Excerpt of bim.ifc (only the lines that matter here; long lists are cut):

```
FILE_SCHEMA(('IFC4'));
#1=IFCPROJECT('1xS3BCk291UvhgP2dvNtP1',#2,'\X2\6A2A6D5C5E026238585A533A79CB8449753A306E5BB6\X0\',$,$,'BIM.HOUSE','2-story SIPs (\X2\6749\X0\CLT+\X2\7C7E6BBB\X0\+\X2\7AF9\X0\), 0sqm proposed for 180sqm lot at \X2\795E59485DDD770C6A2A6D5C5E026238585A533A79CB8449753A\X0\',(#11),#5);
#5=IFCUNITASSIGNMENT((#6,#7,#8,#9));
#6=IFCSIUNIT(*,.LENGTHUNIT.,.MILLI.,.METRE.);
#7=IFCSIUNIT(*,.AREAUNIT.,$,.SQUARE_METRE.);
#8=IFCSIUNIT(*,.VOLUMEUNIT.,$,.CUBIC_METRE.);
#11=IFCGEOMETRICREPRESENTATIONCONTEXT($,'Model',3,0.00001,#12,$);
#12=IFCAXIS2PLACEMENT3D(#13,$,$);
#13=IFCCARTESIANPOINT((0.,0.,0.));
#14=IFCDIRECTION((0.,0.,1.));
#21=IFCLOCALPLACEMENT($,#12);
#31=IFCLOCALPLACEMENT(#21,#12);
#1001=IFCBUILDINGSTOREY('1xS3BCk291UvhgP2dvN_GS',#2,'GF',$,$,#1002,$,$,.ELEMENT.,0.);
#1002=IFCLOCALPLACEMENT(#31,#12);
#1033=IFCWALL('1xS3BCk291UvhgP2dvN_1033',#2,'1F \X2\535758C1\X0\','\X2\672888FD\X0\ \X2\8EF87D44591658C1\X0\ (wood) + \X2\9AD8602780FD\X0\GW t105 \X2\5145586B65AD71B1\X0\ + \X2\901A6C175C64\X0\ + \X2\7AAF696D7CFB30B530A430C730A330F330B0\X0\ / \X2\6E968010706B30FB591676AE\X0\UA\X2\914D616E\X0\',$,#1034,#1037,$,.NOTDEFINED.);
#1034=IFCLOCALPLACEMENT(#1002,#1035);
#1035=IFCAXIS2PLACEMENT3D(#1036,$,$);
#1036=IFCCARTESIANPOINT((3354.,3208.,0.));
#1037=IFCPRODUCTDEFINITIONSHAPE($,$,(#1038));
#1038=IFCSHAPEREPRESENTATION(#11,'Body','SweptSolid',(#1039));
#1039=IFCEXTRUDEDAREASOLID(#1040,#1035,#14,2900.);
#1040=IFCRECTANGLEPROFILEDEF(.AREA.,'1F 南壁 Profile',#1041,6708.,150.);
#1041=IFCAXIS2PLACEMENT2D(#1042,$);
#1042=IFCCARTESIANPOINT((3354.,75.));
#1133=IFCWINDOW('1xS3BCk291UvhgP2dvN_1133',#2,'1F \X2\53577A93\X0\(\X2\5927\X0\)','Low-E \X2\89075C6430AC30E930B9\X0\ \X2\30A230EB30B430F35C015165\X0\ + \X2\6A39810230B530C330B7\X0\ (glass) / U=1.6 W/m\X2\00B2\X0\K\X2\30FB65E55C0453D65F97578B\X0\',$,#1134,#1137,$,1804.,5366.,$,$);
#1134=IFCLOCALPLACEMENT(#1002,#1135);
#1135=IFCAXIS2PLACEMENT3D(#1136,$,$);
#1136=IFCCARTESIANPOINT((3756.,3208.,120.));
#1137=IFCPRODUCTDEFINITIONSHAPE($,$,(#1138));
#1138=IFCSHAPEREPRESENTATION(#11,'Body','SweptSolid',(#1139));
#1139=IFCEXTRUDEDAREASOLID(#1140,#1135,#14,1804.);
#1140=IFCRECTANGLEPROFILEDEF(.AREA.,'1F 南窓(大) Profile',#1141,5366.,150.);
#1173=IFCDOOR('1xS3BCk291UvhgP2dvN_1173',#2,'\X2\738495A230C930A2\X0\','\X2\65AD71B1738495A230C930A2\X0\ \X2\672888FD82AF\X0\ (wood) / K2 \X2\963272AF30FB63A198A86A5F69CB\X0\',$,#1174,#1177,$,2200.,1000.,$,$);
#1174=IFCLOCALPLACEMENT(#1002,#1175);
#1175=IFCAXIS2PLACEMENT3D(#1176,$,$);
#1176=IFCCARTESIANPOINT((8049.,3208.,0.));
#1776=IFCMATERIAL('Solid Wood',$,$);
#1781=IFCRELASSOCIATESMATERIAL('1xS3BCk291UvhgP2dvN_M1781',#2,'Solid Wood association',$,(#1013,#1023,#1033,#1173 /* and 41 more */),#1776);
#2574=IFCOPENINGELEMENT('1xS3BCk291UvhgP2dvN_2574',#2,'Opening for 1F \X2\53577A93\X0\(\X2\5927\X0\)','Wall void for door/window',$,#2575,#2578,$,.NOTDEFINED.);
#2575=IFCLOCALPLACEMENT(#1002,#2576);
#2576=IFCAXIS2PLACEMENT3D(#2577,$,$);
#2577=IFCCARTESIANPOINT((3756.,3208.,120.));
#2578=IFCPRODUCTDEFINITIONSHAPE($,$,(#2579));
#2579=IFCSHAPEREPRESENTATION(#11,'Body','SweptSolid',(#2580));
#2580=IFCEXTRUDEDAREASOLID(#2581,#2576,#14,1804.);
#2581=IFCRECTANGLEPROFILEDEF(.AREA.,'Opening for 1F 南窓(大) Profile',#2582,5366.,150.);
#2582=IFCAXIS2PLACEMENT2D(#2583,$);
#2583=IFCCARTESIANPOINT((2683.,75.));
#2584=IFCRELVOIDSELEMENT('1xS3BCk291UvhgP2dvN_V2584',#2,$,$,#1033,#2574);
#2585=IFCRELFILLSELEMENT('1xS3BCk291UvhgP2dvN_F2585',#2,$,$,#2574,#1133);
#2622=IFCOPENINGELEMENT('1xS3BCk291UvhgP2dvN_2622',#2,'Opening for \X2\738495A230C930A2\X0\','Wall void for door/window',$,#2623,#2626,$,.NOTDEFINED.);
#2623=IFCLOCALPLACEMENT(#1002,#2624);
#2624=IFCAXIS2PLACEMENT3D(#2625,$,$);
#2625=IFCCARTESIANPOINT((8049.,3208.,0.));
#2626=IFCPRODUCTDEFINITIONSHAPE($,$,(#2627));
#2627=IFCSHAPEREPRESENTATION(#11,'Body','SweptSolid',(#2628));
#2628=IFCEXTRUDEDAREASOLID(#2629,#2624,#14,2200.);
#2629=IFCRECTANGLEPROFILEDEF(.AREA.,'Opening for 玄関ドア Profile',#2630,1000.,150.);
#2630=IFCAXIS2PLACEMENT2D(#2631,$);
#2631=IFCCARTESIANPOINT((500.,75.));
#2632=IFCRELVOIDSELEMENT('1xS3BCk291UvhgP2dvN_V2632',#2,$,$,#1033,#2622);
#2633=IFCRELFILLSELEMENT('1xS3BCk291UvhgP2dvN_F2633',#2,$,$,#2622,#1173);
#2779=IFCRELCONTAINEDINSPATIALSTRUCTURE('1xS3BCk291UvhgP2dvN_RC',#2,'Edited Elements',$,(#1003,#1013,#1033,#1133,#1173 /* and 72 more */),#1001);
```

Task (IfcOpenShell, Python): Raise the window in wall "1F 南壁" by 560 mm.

```python
import numpy as np
import ifcopenshell
import ifcopenshell.api.geometry
import ifcopenshell.util.placement
import ifcopenshell.util.unit

model = ifcopenshell.open("bim.ifc")
unit_scale = ifcopenshell.util.unit.calculate_unit_scale(model)

window = model.by_id(1133)
opening = window.FillsVoids[0].RelatingOpeningElement
dz = 560.0

shift = np.array([0.0, 0.0, dz])
# The window is not placed relative to its opening, so move both.
for product in (opening, window):
    matrix = ifcopenshell.util.placement.get_local_placement(product.ObjectPlacement)
    matrix[:3, 3] += shift
    ifcopenshell.api.geometry.edit_object_placement(model, product=product, matrix=matrix, is_si=False)

print(f"moved by {dz * unit_scale:+.3f} m")

model.write("bim_updated.ifc")
```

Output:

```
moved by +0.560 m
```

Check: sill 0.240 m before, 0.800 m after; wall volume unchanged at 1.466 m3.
